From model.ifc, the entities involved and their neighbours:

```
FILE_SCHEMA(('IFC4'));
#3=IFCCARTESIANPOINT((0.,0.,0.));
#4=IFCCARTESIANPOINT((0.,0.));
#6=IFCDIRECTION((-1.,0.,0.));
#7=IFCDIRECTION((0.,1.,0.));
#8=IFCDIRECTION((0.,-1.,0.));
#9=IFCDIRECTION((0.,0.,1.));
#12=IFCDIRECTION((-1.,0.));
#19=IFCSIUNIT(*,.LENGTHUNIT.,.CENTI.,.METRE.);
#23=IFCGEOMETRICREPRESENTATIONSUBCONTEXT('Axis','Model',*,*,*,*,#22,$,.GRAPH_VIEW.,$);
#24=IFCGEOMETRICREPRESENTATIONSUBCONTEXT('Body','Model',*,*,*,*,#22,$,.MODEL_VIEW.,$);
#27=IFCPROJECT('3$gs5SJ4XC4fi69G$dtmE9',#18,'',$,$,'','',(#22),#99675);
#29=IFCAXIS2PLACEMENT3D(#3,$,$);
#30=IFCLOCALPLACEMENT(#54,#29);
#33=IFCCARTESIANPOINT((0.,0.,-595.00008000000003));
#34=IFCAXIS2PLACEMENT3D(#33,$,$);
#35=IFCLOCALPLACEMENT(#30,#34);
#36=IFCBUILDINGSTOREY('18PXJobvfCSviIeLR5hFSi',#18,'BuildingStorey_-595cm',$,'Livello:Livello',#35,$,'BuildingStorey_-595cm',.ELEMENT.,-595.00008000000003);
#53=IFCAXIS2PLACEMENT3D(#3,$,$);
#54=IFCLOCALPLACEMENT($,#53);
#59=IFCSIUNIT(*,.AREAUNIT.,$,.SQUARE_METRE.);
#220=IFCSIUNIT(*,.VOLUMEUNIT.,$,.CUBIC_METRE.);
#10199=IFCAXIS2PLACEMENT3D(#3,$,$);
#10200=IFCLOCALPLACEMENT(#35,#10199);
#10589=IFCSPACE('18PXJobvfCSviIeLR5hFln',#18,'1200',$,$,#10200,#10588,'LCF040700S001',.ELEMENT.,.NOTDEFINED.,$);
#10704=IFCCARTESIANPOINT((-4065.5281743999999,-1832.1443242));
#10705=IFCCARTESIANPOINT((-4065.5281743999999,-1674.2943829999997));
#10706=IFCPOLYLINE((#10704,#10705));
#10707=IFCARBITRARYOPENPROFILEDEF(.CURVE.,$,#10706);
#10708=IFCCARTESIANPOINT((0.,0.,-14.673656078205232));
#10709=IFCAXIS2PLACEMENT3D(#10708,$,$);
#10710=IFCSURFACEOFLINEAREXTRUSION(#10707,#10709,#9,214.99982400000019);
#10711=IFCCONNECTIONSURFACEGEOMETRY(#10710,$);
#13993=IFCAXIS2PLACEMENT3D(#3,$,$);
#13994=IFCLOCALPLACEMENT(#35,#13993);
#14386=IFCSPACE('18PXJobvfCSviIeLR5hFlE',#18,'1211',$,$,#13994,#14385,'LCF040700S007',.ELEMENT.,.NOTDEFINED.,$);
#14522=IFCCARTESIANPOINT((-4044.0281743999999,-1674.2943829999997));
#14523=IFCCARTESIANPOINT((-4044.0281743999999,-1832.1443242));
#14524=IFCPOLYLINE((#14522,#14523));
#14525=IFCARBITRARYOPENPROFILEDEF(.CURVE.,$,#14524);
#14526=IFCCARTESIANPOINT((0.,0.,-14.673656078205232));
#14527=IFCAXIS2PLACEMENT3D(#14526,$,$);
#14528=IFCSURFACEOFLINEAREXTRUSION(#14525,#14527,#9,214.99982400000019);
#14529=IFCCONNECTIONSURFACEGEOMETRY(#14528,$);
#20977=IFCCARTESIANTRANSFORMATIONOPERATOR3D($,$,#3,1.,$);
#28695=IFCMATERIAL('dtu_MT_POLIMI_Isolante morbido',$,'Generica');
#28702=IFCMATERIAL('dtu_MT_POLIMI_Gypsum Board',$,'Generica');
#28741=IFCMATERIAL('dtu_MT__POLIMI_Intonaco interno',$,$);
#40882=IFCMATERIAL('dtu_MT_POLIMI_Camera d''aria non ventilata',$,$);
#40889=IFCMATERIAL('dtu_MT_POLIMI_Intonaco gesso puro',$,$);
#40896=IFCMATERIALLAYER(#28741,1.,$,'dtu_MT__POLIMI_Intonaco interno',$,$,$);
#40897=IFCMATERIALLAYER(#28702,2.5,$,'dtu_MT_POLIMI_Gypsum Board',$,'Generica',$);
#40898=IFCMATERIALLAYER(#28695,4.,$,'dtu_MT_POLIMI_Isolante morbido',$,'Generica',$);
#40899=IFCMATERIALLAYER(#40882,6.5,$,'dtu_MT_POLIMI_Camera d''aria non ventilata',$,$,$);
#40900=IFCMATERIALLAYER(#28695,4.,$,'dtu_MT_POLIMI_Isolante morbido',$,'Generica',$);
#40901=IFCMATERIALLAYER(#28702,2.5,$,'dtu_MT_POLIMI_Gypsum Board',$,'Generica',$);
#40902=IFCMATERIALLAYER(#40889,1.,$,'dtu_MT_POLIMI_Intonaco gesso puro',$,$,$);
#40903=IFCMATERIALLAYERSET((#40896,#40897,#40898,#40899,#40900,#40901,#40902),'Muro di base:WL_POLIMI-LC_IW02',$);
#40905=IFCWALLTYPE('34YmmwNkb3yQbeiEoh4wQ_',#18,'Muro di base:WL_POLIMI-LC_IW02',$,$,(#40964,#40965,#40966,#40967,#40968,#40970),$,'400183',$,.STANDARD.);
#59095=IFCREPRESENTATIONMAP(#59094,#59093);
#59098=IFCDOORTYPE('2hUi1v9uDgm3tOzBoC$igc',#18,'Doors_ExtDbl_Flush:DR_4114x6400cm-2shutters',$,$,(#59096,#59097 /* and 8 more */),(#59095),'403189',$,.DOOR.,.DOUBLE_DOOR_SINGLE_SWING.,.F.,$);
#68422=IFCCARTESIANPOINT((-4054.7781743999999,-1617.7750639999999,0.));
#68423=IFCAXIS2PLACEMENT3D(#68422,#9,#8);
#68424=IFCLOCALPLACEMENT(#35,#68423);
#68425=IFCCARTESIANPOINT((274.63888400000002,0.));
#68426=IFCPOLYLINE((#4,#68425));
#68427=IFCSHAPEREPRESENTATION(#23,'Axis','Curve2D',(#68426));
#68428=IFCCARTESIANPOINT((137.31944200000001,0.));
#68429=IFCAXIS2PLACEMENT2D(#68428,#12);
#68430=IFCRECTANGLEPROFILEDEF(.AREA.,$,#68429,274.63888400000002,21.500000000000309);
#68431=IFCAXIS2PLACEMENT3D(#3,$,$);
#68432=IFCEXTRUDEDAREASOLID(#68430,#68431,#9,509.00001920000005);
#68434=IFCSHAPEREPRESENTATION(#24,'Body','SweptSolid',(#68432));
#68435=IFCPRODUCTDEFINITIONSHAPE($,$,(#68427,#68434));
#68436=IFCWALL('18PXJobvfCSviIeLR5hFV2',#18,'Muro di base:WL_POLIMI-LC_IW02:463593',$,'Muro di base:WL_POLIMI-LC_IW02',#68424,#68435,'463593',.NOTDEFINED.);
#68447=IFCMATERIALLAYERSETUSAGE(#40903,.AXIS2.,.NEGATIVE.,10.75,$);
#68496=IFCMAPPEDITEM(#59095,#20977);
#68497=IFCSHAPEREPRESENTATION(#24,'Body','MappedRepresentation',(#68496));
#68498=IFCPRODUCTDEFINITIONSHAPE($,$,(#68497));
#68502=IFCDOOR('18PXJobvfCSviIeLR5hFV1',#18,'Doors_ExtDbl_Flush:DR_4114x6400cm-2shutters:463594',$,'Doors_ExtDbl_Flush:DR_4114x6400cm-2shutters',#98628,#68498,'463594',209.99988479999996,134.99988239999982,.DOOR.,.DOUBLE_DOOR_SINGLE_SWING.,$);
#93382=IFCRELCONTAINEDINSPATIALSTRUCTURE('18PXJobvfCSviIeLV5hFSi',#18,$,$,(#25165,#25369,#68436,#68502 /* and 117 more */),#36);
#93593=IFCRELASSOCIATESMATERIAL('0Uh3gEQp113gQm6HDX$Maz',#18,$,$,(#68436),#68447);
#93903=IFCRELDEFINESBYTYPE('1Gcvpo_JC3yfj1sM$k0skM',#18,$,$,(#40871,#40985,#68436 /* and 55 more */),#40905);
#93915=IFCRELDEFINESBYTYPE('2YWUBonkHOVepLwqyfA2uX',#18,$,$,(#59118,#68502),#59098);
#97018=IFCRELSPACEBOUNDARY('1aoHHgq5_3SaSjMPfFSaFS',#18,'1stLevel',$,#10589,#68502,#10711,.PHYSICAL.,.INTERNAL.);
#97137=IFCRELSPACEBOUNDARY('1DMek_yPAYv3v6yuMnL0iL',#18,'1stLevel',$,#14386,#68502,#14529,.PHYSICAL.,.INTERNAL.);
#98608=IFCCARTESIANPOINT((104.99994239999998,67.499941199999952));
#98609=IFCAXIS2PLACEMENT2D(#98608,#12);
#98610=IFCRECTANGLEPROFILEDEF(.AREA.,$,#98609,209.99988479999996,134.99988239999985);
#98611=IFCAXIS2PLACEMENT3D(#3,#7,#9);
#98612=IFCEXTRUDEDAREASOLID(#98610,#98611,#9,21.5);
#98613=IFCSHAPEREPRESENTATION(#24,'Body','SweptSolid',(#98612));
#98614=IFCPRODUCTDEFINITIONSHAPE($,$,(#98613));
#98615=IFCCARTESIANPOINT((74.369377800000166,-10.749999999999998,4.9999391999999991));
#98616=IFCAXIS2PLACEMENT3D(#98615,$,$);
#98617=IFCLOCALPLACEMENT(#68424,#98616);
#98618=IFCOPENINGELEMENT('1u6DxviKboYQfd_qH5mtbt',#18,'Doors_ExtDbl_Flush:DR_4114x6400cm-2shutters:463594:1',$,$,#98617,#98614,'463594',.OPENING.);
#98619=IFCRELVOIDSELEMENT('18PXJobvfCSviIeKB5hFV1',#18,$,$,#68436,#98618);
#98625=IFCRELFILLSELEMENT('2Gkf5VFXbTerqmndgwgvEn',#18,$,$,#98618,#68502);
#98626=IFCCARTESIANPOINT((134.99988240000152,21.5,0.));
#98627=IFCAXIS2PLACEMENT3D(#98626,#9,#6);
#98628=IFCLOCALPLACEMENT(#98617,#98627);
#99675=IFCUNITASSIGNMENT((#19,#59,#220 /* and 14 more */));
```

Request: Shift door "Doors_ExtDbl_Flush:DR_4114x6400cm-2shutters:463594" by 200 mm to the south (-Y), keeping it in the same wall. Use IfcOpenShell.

```python
import numpy as np
import ifcopenshell
import ifcopenshell.api.geometry
import ifcopenshell.util.placement
import ifcopenshell.util.unit

model = ifcopenshell.open("model.ifc")
unit_scale = ifcopenshell.util.unit.calculate_unit_scale(model)

door = model.by_guid("18PXJobvfCSviIeLR5hFV1")
opening = door.FillsVoids[0].RelatingOpeningElement
wall = opening.VoidsElements[0].RelatingBuildingElement

wall_matrix = ifcopenshell.util.placement.get_local_placement(wall.ObjectPlacement)
shift = wall_matrix[:3, 0] * 0.2 / unit_scale
before = ifcopenshell.util.placement.get_local_placement(door.ObjectPlacement)[:3, 3].copy()

# The door is placed relative to its opening, so it follows when the opening moves.
matrix = ifcopenshell.util.placement.get_local_placement(opening.ObjectPlacement)
matrix[:3, 3] += shift
ifcopenshell.api.geometry.edit_object_placement(
    model, product=opening, matrix=matrix, is_si=False, should_transform_children=True
)

# Space boundary surfaces are stored in each space's coordinates; move them too.
for rel in door.ProvidesBoundaries:
    if not rel.ConnectionGeometry:
        continue
    surface = rel.ConnectionGeometry.SurfaceOnRelatingElement
    space_matrix = ifcopenshell.util.placement.get_local_placement(rel.RelatingSpace.ObjectPlacement)
    point = np.array(surface.Position.Location.Coordinates) + space_matrix[:3, :3].T @ shift
    surface.Position = model.createIfcAxis2Placement3D(
        model.createIfcCartesianPoint(point.tolist()), surface.Position.Axis, surface.Position.RefDirection
    )

after = ifcopenshell.util.placement.get_local_placement(door.ObjectPlacement)[:3, 3]
print("door moved by", (after - before).round(3) + 0.0)

model.write("model_edited.ifc")
```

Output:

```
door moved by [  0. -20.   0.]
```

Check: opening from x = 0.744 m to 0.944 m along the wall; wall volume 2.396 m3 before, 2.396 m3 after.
